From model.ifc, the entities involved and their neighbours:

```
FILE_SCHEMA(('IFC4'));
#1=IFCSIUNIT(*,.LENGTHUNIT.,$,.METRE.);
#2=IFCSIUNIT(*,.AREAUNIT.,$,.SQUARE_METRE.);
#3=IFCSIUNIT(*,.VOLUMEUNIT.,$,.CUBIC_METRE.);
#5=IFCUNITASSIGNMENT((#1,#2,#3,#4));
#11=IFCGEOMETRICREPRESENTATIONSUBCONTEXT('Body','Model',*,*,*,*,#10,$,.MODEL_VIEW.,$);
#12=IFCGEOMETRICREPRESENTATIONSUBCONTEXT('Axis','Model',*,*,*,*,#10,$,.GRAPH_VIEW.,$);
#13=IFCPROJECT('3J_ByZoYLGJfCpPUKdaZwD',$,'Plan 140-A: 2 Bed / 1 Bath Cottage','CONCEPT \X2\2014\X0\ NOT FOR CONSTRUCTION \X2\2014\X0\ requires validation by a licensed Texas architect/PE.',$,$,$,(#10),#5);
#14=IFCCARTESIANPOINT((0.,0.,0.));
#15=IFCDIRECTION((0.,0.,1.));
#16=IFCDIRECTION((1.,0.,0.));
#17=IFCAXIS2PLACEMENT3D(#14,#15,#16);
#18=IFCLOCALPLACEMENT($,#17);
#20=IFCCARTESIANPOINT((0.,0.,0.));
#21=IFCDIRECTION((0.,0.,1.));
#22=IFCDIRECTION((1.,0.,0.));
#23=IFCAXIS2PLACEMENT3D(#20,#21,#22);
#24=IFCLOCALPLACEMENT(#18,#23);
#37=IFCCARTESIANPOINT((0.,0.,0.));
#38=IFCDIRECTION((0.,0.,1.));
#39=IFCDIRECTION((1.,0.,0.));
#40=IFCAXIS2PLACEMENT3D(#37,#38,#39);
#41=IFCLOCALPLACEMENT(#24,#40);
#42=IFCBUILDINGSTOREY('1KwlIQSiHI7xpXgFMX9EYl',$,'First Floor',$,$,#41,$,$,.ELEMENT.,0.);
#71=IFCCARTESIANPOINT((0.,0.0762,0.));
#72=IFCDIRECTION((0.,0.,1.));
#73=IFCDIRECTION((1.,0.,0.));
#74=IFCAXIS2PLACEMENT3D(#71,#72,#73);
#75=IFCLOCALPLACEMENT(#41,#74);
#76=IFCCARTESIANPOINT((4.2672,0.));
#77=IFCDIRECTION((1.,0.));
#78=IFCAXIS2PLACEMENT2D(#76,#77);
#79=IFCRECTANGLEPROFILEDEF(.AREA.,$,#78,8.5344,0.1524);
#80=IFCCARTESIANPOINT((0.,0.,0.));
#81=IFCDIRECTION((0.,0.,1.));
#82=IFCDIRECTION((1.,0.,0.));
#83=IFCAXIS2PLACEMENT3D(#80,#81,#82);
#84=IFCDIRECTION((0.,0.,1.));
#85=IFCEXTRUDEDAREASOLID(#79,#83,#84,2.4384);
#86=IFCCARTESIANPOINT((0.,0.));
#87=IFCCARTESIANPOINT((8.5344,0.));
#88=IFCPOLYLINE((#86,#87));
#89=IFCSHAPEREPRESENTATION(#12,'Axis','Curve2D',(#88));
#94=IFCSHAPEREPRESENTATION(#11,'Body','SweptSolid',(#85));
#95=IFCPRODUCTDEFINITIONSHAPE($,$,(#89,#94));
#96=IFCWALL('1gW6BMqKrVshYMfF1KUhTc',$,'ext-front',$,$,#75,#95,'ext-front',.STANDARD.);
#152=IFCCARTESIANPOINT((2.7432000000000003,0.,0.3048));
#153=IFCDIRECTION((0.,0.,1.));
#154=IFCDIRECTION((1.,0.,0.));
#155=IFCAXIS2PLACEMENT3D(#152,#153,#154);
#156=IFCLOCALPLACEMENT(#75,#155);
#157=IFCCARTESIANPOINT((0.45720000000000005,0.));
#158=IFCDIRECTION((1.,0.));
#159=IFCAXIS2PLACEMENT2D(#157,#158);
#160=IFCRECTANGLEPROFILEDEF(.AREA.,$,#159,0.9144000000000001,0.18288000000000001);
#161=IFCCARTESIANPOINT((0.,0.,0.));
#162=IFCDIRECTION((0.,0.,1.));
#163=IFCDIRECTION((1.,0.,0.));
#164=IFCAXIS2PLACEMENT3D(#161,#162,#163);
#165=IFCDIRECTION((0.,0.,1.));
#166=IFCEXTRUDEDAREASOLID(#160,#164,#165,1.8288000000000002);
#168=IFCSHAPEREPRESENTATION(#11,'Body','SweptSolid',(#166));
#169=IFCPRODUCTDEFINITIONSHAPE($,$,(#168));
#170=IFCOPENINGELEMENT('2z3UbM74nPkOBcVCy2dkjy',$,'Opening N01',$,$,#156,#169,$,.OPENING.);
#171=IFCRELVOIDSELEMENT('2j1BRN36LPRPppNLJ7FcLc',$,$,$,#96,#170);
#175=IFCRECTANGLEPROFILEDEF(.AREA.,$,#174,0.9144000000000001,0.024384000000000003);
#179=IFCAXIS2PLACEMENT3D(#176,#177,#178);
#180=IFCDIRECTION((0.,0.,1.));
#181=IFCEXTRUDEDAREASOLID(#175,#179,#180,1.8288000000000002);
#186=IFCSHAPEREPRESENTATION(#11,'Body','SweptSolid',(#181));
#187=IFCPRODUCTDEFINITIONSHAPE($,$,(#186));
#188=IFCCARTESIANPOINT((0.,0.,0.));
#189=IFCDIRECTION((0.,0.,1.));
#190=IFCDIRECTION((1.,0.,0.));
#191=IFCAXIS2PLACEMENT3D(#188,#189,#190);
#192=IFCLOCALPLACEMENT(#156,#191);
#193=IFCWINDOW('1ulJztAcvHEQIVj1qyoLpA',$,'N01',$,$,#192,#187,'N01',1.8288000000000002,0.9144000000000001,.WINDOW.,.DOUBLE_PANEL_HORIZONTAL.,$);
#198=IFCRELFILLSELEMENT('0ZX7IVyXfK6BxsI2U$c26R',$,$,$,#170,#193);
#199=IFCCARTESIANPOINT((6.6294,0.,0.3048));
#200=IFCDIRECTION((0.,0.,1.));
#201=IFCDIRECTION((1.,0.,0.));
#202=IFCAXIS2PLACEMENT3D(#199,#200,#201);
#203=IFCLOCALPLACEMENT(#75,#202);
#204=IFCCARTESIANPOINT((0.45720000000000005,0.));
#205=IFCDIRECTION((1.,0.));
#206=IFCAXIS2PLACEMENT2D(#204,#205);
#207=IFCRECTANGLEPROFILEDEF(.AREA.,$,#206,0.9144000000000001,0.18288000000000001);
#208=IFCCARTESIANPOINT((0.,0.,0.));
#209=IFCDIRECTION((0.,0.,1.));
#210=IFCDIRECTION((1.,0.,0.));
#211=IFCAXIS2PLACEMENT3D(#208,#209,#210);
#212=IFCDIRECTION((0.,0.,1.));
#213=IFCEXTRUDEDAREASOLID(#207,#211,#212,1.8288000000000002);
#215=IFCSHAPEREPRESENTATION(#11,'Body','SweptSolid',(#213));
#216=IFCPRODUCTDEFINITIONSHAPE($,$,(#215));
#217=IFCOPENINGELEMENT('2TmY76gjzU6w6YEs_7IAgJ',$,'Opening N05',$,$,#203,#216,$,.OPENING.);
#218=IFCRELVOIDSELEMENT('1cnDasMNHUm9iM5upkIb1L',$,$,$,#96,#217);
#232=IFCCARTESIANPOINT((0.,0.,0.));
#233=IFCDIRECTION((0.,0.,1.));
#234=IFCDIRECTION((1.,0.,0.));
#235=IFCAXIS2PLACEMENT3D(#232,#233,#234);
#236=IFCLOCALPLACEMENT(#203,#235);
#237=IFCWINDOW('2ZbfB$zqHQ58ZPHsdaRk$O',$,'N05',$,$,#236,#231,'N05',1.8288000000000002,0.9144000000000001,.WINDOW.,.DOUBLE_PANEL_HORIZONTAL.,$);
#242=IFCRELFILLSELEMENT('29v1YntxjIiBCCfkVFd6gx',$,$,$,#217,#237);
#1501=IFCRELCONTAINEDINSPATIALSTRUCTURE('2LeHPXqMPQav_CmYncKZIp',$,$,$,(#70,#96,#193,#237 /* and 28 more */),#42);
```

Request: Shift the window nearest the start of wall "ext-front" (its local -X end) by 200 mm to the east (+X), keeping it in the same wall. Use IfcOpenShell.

```python
import ifcopenshell
import ifcopenshell.api.geometry
import ifcopenshell.util.placement
import ifcopenshell.util.unit

model = ifcopenshell.open("model.ifc")
unit_scale = ifcopenshell.util.unit.calculate_unit_scale(model)

window = model.by_id(193)
opening = window.FillsVoids[0].RelatingOpeningElement
wall = opening.VoidsElements[0].RelatingBuildingElement

wall_matrix = ifcopenshell.util.placement.get_local_placement(wall.ObjectPlacement)
shift = wall_matrix[:3, 0] * 0.2 / unit_scale
before = ifcopenshell.util.placement.get_local_placement(window.ObjectPlacement)[:3, 3].copy()

# The window is placed relative to its opening, so it follows when the opening moves.
matrix = ifcopenshell.util.placement.get_local_placement(opening.ObjectPlacement)
matrix[:3, 3] += shift
ifcopenshell.api.geometry.edit_object_placement(
    model, product=opening, matrix=matrix, is_si=False, should_transform_children=True
)

after = ifcopenshell.util.placement.get_local_placement(window.ObjectPlacement)[:3, 3]
print("window moved by", (after - before).round(3) + 0.0)

model.write("model-out.ifc")
```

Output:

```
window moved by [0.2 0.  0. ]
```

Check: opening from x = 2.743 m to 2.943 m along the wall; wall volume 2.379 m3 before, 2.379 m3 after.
